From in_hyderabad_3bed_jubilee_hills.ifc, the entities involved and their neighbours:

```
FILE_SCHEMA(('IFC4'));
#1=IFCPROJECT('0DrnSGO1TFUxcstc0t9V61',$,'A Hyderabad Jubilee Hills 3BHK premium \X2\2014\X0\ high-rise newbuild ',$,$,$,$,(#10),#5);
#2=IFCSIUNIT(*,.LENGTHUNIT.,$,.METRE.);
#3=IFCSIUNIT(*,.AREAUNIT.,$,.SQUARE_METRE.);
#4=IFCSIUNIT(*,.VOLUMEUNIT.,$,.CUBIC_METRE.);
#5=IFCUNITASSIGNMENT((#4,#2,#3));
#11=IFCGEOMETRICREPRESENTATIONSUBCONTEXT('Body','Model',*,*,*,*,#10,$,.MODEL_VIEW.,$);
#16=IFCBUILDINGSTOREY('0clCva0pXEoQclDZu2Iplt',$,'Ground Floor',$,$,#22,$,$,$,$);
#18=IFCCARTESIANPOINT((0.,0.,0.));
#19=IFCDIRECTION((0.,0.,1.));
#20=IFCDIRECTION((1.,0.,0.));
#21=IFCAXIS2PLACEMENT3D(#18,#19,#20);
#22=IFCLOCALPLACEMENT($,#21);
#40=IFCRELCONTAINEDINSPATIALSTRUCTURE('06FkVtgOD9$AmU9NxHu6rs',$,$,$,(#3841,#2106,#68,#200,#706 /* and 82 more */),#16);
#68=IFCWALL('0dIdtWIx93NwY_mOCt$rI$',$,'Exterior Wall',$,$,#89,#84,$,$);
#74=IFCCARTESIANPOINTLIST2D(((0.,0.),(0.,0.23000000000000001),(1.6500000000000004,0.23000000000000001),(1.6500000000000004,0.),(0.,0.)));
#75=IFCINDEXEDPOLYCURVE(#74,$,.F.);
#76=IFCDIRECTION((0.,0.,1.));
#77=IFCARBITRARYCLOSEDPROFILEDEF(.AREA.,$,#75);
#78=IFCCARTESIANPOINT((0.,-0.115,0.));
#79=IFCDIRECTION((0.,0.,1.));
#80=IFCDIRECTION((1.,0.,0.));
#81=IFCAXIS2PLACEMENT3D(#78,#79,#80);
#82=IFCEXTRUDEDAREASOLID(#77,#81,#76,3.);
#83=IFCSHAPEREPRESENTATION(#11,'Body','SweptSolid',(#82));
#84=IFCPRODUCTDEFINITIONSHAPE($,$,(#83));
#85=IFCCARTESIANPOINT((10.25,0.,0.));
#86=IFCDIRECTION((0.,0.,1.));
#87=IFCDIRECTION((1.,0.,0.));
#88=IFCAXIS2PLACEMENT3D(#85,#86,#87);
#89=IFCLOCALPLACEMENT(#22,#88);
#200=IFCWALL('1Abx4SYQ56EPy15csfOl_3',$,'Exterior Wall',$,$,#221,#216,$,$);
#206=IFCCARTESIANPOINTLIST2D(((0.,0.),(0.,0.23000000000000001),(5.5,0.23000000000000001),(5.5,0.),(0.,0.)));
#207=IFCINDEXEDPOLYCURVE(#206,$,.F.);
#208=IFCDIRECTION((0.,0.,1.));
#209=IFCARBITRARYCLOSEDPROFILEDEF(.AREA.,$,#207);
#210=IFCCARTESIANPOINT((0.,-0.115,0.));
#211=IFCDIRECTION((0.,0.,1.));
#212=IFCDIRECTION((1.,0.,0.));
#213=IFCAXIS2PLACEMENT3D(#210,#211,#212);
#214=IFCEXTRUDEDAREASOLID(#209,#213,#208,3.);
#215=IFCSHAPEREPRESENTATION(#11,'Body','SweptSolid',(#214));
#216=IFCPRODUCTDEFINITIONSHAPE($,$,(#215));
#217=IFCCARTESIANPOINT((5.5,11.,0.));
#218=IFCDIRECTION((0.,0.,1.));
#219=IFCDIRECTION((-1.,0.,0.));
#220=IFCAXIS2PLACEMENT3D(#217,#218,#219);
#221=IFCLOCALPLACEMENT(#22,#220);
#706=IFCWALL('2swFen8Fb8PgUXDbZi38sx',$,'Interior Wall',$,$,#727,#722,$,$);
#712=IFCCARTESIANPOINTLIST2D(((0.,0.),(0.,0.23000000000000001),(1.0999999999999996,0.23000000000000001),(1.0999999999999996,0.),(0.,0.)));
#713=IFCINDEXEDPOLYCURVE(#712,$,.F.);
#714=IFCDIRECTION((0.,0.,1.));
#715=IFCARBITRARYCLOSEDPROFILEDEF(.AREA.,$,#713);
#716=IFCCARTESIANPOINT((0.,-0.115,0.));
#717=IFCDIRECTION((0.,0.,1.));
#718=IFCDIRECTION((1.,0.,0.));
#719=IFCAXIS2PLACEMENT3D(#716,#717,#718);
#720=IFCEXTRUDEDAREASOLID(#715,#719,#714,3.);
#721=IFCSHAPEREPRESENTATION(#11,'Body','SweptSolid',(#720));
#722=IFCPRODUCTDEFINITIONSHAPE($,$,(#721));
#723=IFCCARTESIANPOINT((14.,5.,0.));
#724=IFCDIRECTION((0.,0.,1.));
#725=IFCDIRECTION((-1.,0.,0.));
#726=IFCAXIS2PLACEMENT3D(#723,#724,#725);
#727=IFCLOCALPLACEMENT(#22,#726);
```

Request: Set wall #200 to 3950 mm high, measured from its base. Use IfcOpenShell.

```python
import ifcopenshell
import ifcopenshell.geom
import ifcopenshell.util.representation
import ifcopenshell.util.shape

model = ifcopenshell.open("in_hyderabad_3bed_jubilee_hills.ifc")
settings = ifcopenshell.geom.settings()


def volume(element):
    """Net volume in cubic metres, openings subtracted."""
    shape = ifcopenshell.geom.create_shape(settings, element)
    return ifcopenshell.util.shape.get_volume(shape.geometry)


wall = model.by_id(200)
before = volume(wall)

body = ifcopenshell.util.representation.get_representation(wall, "Model", "Body")
solid = body.Items[0]
old_height = solid.Depth
solid.Depth = 3.95
after = volume(wall)

print(f"height {old_height:g} -> {solid.Depth:g}, volume {before:.3f} -> {after:.3f} m3")

model.write("in_hyderabad_3bed_jubilee_hills_v2.ifc")
```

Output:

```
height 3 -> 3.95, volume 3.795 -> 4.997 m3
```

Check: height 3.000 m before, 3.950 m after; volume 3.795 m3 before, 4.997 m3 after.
